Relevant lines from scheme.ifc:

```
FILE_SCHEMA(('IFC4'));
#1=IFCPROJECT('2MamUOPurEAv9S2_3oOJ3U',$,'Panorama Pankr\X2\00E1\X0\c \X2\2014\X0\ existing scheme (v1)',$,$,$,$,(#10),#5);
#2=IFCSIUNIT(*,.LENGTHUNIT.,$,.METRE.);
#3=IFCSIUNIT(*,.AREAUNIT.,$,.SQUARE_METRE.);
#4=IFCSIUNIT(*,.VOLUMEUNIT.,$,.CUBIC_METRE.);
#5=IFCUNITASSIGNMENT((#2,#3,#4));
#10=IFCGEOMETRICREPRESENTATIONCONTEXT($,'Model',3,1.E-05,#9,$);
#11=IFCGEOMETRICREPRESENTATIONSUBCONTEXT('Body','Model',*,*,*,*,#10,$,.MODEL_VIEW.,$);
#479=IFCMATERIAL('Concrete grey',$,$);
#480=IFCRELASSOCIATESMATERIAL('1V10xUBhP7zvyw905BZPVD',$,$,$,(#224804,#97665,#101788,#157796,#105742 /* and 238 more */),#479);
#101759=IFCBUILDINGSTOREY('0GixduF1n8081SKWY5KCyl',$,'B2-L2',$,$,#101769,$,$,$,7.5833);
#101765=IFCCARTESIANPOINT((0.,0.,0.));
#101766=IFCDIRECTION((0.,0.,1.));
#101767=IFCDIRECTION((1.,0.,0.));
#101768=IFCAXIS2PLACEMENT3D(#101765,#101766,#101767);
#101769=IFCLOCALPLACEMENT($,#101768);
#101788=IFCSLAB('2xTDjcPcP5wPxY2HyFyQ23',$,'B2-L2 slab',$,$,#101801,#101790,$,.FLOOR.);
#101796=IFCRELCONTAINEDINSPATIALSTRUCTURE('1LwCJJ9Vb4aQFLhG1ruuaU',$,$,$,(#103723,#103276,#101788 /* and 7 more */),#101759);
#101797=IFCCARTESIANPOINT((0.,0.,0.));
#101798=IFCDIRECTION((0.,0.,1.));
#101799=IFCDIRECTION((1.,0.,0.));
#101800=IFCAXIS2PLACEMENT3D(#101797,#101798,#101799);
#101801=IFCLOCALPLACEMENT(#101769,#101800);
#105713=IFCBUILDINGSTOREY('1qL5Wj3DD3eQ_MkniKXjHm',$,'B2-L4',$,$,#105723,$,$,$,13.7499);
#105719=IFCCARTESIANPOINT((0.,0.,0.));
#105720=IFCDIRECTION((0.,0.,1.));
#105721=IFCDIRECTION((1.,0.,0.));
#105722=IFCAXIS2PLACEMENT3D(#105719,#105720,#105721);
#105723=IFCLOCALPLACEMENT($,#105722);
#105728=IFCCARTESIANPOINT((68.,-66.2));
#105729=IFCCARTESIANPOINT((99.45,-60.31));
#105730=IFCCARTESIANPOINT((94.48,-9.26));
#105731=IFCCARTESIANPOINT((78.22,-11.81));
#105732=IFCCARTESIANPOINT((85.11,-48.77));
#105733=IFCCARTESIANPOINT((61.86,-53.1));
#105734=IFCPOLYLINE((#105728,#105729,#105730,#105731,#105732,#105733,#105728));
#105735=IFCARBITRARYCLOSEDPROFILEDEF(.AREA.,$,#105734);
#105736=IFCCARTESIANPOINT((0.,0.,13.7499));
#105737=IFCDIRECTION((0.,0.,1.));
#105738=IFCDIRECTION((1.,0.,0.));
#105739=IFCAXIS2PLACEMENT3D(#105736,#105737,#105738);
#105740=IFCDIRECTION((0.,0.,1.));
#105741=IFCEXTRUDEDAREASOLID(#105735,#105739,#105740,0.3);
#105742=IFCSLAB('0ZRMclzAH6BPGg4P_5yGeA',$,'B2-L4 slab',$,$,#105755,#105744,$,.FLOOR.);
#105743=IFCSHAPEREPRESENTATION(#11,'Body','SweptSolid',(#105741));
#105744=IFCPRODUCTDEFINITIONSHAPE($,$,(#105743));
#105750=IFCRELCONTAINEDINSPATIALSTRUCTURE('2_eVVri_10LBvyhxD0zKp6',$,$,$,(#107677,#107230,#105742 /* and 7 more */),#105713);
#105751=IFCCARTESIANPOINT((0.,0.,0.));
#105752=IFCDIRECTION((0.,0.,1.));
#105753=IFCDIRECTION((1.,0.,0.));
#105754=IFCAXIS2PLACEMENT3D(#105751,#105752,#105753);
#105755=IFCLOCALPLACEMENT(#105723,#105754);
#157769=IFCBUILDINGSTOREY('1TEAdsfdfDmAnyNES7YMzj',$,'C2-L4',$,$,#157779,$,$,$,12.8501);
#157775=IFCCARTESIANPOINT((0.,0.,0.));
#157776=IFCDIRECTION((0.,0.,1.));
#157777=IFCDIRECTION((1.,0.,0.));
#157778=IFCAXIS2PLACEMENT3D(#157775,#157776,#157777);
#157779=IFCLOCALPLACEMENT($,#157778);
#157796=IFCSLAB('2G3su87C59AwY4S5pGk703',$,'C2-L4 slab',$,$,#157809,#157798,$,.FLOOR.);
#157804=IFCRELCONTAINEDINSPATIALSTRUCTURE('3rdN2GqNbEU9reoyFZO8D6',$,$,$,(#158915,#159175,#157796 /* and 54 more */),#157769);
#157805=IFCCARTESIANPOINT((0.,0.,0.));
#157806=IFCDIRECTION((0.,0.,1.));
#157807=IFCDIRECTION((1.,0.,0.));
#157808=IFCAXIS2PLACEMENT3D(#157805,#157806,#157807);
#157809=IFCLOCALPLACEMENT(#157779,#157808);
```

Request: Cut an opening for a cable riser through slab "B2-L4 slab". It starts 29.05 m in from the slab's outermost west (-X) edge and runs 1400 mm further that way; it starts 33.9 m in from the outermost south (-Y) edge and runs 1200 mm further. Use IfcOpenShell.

```python
import numpy as np
import ifcopenshell
import ifcopenshell.api.feature
import ifcopenshell.api.geometry
import ifcopenshell.api.root
import ifcopenshell.geom
import ifcopenshell.util.placement
import ifcopenshell.util.representation
import ifcopenshell.util.shape
import ifcopenshell.util.unit

model = ifcopenshell.open("scheme.ifc")
unit_scale = ifcopenshell.util.unit.calculate_unit_scale(model)
settings = ifcopenshell.geom.settings()


def volume(element):
    """Net volume in cubic metres, openings subtracted."""
    shape = ifcopenshell.geom.create_shape(settings, element)
    return ifcopenshell.util.shape.get_volume(shape.geometry)


slab = model.by_id(105742)
before = volume(slab)

# Extent in the slab's own axes, in metres. The edges named are its -X and -Y sides.
slab_shape = ifcopenshell.geom.create_shape(settings, slab)
vertices = ifcopenshell.util.shape.get_vertices(slab_shape.geometry)
x_min, y_min, bottom = vertices.min(axis=0)
top = vertices[:, 2].max()

opening = ifcopenshell.api.root.create_entity(model, ifc_class="IfcOpeningElement", name="Cable riser opening", predefined_type="OPENING")
context = ifcopenshell.util.representation.get_context(model, "Model", "Body", "MODEL_VIEW")
width, depth = 1.4, 1.2
outline = [(0.0, 0.0), (width, 0.0), (width, depth), (0.0, depth), (0.0, 0.0)]
# Overshoot both faces by 50 mm so the cut is clean.
shape = ifcopenshell.api.geometry.add_slab_representation(
    model, context=context, depth=top - bottom + 0.1, polyline=outline
)
ifcopenshell.api.geometry.assign_representation(model, product=opening, representation=shape)

matrix = ifcopenshell.util.placement.get_local_placement(slab.ObjectPlacement)
matrix[:, 3] = matrix @ np.append(np.array([x_min + 29.05, y_min + 33.9, bottom - 0.05]) / unit_scale, 1.0)
ifcopenshell.api.geometry.edit_object_placement(model, product=opening, matrix=matrix, is_si=False)
ifcopenshell.api.feature.add_feature(model, feature=opening, element=slab)

after = volume(slab)

print(f"slab volume {before:.3f} -> {after:.3f} m3")

model.write("scheme_updated.ifc")
```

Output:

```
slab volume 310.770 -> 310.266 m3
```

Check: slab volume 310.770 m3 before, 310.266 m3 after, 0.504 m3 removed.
